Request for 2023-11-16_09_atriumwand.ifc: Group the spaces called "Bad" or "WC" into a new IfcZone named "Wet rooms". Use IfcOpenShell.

First a look at what the model holds.

```python
import ifcopenshell

model = ifcopenshell.open("2023-11-16_09_atriumwand.ifc")
print(model.schema)
seen = {}
for space in model.by_type("IfcSpace"):
    seen[space.LongName] = seen.get(space.LongName, 0) + 1
for name, count in sorted(seen.items(), key=str):
    print(count, "x", name)
print("zones:", [z.Name for z in model.by_type("IfcZone")][:20])
```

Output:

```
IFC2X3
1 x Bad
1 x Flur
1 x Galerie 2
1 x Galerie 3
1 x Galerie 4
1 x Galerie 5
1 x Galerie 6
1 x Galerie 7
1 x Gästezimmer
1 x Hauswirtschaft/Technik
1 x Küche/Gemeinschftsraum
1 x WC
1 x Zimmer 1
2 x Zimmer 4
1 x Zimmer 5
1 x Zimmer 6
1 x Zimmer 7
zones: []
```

```python
import ifcopenshell
import ifcopenshell.api.group
import ifcopenshell.api.root

model = ifcopenshell.open("2023-11-16_09_atriumwand.ifc")

names = {"Bad", "WC"}
spaces = [s for s in model.by_type("IfcSpace") if s.LongName in names]

zone = ifcopenshell.api.root.create_entity(model, ifc_class="IfcZone", name="Wet rooms")
ifcopenshell.api.group.assign_group(model, products=spaces, group=zone)
print(len(spaces), "spaces in", zone.Name)

model.write("2023-11-16_09_atriumwand-out.ifc")
```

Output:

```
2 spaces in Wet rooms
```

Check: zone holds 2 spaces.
